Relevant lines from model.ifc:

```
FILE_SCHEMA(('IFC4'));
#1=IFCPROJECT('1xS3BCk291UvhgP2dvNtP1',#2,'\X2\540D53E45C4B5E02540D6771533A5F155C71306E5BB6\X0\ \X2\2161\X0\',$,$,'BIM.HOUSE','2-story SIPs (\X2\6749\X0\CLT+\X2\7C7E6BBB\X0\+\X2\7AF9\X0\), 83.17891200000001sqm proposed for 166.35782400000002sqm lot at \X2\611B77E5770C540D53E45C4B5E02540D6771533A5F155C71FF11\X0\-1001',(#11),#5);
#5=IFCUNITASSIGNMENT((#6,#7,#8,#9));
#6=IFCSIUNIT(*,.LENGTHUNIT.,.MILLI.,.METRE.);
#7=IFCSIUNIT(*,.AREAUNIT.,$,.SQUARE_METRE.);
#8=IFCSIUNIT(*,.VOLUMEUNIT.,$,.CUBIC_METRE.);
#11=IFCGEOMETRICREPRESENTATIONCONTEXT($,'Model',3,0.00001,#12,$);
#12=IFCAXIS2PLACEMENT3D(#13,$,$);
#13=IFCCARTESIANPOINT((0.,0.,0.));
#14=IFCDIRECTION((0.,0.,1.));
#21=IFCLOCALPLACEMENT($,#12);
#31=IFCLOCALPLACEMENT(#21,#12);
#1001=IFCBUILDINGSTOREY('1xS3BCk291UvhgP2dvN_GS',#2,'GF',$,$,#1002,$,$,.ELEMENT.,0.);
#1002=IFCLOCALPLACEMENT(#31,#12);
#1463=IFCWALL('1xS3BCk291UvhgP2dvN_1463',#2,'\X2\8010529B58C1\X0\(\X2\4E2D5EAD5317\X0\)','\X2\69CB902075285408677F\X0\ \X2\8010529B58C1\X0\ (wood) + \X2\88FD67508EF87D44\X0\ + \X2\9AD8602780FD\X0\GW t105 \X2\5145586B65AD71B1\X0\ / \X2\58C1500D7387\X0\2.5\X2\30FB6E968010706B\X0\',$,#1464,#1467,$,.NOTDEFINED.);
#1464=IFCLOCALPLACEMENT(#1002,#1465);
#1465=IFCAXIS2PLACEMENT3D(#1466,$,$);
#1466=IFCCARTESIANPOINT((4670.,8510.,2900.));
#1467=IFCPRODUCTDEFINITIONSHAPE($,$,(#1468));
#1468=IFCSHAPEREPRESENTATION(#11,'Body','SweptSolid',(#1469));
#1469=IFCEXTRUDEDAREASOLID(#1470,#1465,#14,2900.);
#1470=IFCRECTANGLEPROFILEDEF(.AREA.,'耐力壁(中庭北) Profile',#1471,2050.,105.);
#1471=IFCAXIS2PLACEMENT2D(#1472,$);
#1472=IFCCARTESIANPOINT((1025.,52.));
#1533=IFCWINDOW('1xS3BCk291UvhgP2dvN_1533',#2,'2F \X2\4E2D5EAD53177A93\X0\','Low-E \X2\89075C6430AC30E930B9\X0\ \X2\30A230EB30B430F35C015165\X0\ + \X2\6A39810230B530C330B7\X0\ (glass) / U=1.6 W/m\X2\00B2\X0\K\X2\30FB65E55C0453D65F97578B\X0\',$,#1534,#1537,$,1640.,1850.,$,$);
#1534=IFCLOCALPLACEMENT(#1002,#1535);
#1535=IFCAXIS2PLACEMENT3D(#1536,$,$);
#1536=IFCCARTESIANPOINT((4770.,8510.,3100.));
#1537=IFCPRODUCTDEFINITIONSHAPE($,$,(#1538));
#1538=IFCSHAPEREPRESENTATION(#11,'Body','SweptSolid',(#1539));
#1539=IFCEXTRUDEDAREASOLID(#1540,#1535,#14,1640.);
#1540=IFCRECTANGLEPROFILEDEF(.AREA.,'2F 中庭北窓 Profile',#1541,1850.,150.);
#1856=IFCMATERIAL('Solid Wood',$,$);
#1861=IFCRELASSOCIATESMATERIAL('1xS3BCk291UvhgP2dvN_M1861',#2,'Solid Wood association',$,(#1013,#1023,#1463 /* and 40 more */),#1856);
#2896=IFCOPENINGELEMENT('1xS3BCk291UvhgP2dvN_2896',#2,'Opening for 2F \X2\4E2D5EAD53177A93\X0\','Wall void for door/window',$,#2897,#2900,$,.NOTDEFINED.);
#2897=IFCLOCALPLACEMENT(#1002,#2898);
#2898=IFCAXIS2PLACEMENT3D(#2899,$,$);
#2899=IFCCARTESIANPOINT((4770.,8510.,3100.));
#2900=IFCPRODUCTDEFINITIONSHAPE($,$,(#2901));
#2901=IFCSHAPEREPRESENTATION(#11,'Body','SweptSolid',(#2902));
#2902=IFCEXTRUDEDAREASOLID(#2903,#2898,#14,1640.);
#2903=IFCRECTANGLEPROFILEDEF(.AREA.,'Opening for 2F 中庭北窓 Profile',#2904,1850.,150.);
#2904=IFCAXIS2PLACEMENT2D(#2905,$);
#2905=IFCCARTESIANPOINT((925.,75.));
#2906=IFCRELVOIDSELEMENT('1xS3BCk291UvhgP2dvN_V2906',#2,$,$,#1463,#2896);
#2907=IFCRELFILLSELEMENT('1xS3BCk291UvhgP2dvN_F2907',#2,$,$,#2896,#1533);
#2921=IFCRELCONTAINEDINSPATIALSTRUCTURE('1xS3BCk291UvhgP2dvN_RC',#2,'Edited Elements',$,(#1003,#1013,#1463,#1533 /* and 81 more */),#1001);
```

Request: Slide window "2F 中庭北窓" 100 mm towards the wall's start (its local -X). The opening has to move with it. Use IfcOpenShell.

```python
import ifcopenshell
import ifcopenshell.api.geometry
import ifcopenshell.util.placement

model = ifcopenshell.open("model.ifc")

window = model.by_guid("1xS3BCk291UvhgP2dvN_1533")
opening = window.FillsVoids[0].RelatingOpeningElement
wall = opening.VoidsElements[0].RelatingBuildingElement

wall_matrix = ifcopenshell.util.placement.get_local_placement(wall.ObjectPlacement)
shift = wall_matrix[:3, 0] * -100.0
before = ifcopenshell.util.placement.get_local_placement(window.ObjectPlacement)[:3, 3].copy()

# The window is not placed relative to its opening, so move both.
for product in (opening, window):
    matrix = ifcopenshell.util.placement.get_local_placement(product.ObjectPlacement)
    matrix[:3, 3] += shift
    ifcopenshell.api.geometry.edit_object_placement(model, product=product, matrix=matrix, is_si=False)

after = ifcopenshell.util.placement.get_local_placement(window.ObjectPlacement)[:3, 3]
print("window moved by", (after - before).round(3) + 0.0)

model.write("model_rev.ifc")
```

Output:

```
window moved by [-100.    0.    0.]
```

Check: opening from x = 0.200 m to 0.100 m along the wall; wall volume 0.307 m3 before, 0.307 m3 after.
